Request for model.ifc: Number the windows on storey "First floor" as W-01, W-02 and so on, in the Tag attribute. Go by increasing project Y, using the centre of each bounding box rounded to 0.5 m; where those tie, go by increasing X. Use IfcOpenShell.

First a look at what the model holds.

```python
import ifcopenshell
import ifcopenshell.util.element
import ifcopenshell.util.placement

model = ifcopenshell.open("model.ifc")
print(model.schema)
storey = next(s for s in model.by_type("IfcBuildingStorey") if s.Name == "First floor")
windows = [e for e in ifcopenshell.util.element.get_decomposition(storey) if e.is_a("IfcWindow")]
for e in sorted(windows, key=lambda e: e.id()):
    origin = ifcopenshell.util.placement.get_local_placement(e.ObjectPlacement)[:3, 3]
    print(e.id(), e.Tag, e.Name, origin.round(2) + 0.0, sep=" | ")
```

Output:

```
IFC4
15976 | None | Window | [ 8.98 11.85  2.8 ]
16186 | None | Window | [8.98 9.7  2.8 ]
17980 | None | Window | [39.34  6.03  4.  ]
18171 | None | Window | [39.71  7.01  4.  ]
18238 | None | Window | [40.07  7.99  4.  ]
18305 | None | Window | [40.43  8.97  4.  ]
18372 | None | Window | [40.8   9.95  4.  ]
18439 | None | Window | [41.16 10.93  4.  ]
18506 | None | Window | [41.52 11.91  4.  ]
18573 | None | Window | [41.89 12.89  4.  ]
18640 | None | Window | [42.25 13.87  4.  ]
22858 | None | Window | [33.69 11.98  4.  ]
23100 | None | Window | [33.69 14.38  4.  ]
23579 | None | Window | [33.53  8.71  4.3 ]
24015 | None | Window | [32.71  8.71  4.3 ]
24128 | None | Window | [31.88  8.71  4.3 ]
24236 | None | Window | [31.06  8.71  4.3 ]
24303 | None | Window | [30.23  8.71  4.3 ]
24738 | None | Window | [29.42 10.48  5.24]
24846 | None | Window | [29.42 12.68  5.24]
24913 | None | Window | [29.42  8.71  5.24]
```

```python
import ifcopenshell
import ifcopenshell.geom
import ifcopenshell.util.element
import ifcopenshell.util.shape

model = ifcopenshell.open("model.ifc")
settings = ifcopenshell.geom.settings()
settings.set("use-world-coords", True)


def centre(element):
    shape = ifcopenshell.geom.create_shape(settings, element)
    return ifcopenshell.util.shape.get_bbox_centroid(shape.geometry)


storey = next(s for s in model.by_type("IfcBuildingStorey") if s.Name == "First floor")
windows = [e for e in ifcopenshell.util.element.get_decomposition(storey) if e.is_a("IfcWindow")]

# Insertion points can sit at a corner or the storey origin, so sort by the geometry (in metres).
centres = {e: centre(e) for e in windows}
windows.sort(key=lambda e: (round(centres[e][1] / 0.5), centres[e][0]))

for i, e in enumerate(windows, start=1):
    number = f"W-{i:02d}"
    e.Tag = number
    print(e.id(), number)

model.write("model_v2.ifc")
```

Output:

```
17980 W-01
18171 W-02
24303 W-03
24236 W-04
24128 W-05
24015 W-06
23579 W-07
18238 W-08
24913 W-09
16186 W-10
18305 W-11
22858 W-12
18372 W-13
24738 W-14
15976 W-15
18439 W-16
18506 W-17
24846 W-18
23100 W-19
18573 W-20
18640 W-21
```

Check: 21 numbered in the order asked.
